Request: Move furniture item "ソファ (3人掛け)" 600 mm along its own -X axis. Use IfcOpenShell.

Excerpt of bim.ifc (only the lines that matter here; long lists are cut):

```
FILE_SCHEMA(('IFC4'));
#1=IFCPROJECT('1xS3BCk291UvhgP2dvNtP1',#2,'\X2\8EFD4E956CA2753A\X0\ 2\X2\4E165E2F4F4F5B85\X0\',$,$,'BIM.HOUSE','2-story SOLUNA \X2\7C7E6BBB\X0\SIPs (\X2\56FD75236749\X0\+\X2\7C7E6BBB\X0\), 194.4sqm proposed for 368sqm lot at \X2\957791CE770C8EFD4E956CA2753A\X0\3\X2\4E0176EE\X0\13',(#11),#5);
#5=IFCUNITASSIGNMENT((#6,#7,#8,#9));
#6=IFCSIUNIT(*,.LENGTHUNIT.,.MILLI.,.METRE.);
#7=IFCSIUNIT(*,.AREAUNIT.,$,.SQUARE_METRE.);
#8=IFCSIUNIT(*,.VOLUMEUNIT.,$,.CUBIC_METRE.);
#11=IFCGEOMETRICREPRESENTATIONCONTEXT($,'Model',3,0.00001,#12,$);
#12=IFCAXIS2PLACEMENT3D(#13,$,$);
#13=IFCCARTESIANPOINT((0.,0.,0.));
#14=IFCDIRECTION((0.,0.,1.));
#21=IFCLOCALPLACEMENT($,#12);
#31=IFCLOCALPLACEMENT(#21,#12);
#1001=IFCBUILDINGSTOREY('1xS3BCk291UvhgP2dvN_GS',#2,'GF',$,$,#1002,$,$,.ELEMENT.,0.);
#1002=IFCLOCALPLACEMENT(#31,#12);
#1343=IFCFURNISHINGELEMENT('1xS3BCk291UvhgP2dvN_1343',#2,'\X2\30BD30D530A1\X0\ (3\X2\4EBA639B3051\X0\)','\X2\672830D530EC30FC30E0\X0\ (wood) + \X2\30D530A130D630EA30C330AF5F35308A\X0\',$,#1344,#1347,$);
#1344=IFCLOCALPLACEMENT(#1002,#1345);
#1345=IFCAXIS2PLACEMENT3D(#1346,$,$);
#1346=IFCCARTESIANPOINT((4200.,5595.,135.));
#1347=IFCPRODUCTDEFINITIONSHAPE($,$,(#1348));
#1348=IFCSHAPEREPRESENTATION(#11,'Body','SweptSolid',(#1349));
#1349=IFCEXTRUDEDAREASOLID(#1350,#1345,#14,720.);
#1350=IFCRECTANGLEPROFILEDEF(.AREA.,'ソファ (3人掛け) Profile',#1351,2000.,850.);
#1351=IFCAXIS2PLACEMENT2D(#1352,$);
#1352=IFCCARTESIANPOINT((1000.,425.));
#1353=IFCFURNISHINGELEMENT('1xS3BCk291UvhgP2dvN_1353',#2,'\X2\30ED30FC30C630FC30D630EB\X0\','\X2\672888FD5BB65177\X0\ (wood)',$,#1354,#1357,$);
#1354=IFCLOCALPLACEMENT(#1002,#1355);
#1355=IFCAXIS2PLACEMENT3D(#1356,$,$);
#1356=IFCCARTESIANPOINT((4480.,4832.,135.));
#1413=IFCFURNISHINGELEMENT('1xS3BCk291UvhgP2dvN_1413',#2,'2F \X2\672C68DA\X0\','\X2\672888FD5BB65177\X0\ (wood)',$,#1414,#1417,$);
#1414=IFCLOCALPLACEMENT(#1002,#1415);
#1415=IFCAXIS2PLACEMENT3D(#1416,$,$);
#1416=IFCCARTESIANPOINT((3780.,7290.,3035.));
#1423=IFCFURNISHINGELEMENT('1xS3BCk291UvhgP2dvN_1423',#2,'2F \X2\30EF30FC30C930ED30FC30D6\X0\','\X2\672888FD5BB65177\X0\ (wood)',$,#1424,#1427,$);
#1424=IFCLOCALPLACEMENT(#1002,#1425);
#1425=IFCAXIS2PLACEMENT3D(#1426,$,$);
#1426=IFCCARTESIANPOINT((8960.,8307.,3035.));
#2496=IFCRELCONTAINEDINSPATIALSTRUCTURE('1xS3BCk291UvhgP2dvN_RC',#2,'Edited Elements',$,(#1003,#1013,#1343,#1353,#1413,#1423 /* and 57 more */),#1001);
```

```python
import ifcopenshell
import ifcopenshell.api.geometry
import ifcopenshell.util.placement
import ifcopenshell.util.unit

model = ifcopenshell.open("bim.ifc")
unit_scale = ifcopenshell.util.unit.calculate_unit_scale(model)

item = model.by_guid("1xS3BCk291UvhgP2dvN_1343")
matrix = ifcopenshell.util.placement.get_local_placement(item.ObjectPlacement)
matrix[:3, 3] -= matrix[:3, 0] * 0.6 / unit_scale
ifcopenshell.api.geometry.edit_object_placement(model, product=item, matrix=matrix, is_si=False)

print(ifcopenshell.util.placement.get_local_placement(item.ObjectPlacement).round(3) + 0.0)

model.write("bim_v2.ifc")
```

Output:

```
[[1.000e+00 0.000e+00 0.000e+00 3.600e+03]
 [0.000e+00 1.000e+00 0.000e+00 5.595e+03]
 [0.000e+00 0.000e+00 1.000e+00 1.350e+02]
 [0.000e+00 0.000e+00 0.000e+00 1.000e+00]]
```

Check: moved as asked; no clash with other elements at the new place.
